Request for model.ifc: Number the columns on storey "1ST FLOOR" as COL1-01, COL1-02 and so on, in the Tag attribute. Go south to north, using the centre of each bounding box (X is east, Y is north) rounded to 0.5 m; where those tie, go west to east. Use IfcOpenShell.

First a look at what the model holds.

```python
import ifcopenshell
import ifcopenshell.util.element
import ifcopenshell.util.placement

model = ifcopenshell.open("model.ifc")
print(model.schema)
storey = next(s for s in model.by_type("IfcBuildingStorey") if s.Name == "1ST FLOOR")
columns = [e for e in ifcopenshell.util.element.get_decomposition(storey) if e.is_a("IfcColumn")]
for e in sorted(columns, key=lambda e: e.id()):
    origin = ifcopenshell.util.placement.get_local_placement(e.ObjectPlacement)[:3, 3]
    print(e.id(), e.Tag, e.Name, origin.round(2) + 0.0, sep=" | ")
```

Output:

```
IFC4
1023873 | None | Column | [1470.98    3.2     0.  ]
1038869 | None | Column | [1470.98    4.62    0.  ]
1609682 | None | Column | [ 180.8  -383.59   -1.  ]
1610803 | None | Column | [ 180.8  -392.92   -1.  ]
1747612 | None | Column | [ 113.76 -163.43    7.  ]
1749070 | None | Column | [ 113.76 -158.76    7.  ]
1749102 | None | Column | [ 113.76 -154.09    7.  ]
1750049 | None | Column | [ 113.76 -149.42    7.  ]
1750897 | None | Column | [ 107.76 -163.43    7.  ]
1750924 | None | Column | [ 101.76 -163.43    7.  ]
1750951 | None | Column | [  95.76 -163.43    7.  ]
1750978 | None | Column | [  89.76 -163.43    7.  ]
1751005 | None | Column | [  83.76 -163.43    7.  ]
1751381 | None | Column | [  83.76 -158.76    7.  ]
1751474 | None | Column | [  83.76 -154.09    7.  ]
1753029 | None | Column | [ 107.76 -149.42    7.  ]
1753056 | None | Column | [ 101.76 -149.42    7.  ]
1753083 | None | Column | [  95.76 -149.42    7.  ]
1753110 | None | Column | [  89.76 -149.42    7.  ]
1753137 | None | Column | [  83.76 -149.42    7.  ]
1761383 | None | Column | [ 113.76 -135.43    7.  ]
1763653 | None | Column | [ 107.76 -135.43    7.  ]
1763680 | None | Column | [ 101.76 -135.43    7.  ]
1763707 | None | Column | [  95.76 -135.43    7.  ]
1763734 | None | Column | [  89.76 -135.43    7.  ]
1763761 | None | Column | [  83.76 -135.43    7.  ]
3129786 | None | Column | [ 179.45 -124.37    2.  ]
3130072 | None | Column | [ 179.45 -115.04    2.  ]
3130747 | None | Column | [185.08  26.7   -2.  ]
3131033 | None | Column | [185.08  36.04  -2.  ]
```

```python
import ifcopenshell
import ifcopenshell.geom
import ifcopenshell.util.element
import ifcopenshell.util.shape

model = ifcopenshell.open("model.ifc")
settings = ifcopenshell.geom.settings()
settings.set("use-world-coords", True)


def centre(element):
    shape = ifcopenshell.geom.create_shape(settings, element)
    return ifcopenshell.util.shape.get_bbox_centroid(shape.geometry)


storey = next(s for s in model.by_type("IfcBuildingStorey") if s.Name == "1ST FLOOR")
columns = [e for e in ifcopenshell.util.element.get_decomposition(storey) if e.is_a("IfcColumn")]

# Insertion points can sit at a corner or the storey origin, so sort by the geometry (in metres).
centres = {e: centre(e) for e in columns}
columns.sort(key=lambda e: (round(centres[e][1] / 0.5), centres[e][0]))

for i, e in enumerate(columns, start=1):
    number = f"COL1-{i:02d}"
    e.Tag = number
    print(e.id(), number)

model.write("model-out.ifc")
```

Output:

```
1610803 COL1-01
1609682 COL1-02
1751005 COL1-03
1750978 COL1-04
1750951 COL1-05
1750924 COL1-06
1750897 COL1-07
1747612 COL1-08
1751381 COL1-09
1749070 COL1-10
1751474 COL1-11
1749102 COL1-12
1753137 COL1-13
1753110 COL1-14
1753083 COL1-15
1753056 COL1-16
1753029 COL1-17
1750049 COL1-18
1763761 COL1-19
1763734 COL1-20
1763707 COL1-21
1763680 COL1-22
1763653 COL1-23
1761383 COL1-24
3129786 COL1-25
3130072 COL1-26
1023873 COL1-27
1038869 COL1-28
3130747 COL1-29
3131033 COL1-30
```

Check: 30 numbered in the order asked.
